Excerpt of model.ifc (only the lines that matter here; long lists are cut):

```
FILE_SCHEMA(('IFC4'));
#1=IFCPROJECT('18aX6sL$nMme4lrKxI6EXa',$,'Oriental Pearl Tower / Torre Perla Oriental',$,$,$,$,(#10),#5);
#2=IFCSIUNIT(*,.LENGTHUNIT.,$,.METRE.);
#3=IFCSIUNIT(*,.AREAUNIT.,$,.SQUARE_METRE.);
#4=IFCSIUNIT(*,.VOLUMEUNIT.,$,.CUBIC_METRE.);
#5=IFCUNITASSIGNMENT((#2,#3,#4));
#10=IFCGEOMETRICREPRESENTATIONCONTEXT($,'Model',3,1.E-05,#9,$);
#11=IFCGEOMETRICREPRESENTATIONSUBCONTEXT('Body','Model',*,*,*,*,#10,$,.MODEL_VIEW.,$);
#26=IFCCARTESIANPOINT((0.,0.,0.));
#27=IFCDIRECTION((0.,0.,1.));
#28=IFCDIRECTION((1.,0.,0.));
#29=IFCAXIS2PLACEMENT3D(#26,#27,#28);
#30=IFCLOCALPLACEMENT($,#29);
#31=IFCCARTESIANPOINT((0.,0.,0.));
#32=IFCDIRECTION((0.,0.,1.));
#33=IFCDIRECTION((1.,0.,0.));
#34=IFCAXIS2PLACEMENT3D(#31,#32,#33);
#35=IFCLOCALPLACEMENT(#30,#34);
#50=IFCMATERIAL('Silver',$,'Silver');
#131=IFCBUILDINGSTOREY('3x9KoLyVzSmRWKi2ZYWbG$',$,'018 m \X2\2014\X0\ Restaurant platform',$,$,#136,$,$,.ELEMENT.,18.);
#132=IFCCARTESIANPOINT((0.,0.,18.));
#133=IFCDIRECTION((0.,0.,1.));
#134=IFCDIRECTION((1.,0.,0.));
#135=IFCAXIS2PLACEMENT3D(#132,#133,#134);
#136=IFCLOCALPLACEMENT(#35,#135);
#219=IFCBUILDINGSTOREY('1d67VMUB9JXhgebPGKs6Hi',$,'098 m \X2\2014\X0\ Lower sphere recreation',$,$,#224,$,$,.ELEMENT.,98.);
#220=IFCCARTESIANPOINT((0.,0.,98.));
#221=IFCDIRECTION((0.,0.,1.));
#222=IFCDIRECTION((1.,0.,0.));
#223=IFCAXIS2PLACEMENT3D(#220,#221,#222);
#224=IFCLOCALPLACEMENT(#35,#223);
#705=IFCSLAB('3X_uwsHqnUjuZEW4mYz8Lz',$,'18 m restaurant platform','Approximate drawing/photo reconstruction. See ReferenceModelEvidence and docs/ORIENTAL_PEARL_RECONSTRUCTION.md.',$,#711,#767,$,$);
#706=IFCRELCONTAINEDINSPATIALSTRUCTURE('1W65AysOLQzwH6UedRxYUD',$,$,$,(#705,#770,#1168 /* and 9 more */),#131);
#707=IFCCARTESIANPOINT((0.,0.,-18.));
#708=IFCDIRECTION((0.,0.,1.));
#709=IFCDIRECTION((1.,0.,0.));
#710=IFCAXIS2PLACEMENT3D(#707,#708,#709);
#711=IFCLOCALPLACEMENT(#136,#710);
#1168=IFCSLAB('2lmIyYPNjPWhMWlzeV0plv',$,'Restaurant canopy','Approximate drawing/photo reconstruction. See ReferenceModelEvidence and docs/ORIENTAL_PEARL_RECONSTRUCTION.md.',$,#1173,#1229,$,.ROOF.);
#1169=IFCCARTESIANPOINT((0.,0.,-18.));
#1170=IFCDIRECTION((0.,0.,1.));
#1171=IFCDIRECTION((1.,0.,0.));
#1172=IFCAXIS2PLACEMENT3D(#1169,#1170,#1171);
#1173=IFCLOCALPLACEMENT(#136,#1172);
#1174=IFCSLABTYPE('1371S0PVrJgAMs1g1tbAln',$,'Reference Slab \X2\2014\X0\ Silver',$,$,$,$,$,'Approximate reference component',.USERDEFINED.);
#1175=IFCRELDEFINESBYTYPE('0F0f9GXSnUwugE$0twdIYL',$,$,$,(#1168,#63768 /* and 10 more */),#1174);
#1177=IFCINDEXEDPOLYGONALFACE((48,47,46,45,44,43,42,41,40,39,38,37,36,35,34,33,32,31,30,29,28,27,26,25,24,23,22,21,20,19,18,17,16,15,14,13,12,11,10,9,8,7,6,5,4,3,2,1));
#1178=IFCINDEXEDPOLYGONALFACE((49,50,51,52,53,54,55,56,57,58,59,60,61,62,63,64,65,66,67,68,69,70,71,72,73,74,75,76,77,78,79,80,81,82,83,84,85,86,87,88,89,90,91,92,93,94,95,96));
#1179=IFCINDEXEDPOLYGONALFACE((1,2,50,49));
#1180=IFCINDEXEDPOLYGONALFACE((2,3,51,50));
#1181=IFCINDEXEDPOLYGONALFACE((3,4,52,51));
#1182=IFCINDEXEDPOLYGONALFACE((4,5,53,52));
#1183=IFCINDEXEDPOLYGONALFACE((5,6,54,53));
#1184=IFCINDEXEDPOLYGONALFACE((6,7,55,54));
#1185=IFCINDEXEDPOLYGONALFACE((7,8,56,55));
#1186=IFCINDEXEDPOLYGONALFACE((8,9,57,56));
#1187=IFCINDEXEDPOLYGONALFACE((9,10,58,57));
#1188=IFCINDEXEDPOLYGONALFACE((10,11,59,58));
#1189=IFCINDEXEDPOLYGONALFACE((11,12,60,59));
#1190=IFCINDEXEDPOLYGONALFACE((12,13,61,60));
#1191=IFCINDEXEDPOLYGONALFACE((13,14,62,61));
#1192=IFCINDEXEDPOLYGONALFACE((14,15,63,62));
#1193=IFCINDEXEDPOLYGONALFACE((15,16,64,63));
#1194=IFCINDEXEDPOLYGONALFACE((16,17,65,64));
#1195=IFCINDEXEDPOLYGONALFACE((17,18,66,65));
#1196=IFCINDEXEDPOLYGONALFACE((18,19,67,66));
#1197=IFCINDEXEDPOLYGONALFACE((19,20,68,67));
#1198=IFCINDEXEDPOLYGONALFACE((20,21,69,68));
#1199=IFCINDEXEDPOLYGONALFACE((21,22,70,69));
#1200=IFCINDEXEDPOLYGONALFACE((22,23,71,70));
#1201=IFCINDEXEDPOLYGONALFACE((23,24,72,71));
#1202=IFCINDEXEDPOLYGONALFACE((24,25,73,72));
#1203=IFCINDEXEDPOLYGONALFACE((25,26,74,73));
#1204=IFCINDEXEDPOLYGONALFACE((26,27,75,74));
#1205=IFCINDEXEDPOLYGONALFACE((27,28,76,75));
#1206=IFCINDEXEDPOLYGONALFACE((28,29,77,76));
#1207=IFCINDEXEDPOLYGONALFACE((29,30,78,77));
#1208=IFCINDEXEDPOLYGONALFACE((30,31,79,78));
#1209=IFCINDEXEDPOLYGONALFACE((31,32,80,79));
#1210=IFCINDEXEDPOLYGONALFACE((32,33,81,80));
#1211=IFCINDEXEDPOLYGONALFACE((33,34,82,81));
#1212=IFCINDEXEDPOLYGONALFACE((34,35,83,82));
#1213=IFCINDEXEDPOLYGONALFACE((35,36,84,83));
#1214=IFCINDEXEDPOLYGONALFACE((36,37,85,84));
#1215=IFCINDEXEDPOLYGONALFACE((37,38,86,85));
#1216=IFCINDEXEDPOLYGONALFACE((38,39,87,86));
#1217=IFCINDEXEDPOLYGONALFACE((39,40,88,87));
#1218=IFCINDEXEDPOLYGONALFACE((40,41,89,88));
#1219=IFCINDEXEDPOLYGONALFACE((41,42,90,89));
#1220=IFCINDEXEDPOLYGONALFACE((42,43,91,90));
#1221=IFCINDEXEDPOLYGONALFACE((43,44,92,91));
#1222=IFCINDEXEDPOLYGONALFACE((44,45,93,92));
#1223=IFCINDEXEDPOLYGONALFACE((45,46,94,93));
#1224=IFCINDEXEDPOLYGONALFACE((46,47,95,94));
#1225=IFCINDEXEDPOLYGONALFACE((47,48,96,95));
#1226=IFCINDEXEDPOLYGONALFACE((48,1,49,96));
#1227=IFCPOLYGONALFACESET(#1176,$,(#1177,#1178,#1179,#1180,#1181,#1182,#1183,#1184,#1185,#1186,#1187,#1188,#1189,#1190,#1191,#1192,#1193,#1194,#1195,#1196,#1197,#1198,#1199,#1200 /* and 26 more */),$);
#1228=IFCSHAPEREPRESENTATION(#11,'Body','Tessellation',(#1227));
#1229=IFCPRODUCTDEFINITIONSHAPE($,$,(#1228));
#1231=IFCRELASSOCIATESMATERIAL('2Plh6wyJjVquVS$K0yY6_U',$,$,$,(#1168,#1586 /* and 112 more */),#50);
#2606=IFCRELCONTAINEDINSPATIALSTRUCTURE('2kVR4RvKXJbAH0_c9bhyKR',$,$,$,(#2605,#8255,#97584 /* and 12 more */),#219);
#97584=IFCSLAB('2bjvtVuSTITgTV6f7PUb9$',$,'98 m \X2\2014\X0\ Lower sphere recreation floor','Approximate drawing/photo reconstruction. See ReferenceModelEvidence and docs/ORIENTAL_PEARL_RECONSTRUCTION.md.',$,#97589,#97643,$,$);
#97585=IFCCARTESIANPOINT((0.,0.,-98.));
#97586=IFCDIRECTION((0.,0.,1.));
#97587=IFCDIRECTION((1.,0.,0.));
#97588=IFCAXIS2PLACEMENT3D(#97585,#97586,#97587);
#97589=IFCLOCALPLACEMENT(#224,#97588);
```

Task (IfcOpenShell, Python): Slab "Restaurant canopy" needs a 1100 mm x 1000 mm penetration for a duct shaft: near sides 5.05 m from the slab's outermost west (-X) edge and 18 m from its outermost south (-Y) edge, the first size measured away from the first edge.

```python
import numpy as np
import ifcopenshell
import ifcopenshell.api.feature
import ifcopenshell.api.geometry
import ifcopenshell.api.root
import ifcopenshell.geom
import ifcopenshell.util.placement
import ifcopenshell.util.representation
import ifcopenshell.util.shape
import ifcopenshell.util.unit

model = ifcopenshell.open("model.ifc")
unit_scale = ifcopenshell.util.unit.calculate_unit_scale(model)
settings = ifcopenshell.geom.settings()


def volume(element):
    """Net volume in cubic metres, openings subtracted."""
    shape = ifcopenshell.geom.create_shape(settings, element)
    return ifcopenshell.util.shape.get_volume(shape.geometry)


slab = model.by_guid("2lmIyYPNjPWhMWlzeV0plv")
before = volume(slab)

# Extent in the slab's own axes, in metres. The edges named are its -X and -Y sides.
slab_shape = ifcopenshell.geom.create_shape(settings, slab)
vertices = ifcopenshell.util.shape.get_vertices(slab_shape.geometry)
x_min, y_min, bottom = vertices.min(axis=0)
top = vertices[:, 2].max()

opening = ifcopenshell.api.root.create_entity(model, ifc_class="IfcOpeningElement", name="Duct shaft opening", predefined_type="OPENING")
context = ifcopenshell.util.representation.get_context(model, "Model", "Body", "MODEL_VIEW")
width, depth = 1.1, 1
outline = [(0.0, 0.0), (width, 0.0), (width, depth), (0.0, depth), (0.0, 0.0)]
# Overshoot both faces by 50 mm so the cut is clean.
shape = ifcopenshell.api.geometry.add_slab_representation(
    model, context=context, depth=top - bottom + 0.1, polyline=outline
)
ifcopenshell.api.geometry.assign_representation(model, product=opening, representation=shape)

matrix = ifcopenshell.util.placement.get_local_placement(slab.ObjectPlacement)
matrix[:, 3] = matrix @ np.append(np.array([x_min + 5.05, y_min + 18, bottom - 0.05]) / unit_scale, 1.0)
ifcopenshell.api.geometry.edit_object_placement(model, product=opening, matrix=matrix, is_si=False)
ifcopenshell.api.feature.add_feature(model, feature=opening, element=slab)

after = volume(slab)

print(f"slab volume {before:.3f} -> {after:.3f} m3")

model.write("model_rev.ifc")
```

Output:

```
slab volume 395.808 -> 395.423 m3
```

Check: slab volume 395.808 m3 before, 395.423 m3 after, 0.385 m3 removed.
